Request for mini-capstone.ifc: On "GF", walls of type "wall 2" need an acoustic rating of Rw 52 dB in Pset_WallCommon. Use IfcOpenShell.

First a look at what the model holds.

```python
import ifcopenshell
import ifcopenshell.util.element

model = ifcopenshell.open("mini-capstone.ifc")
print(model.schema)
storey = next(s for s in model.by_type("IfcBuildingStorey") if s.Name == "GF")
walls = [e for e in ifcopenshell.util.element.get_decomposition(storey) if e.is_a("IfcWall")]
seen = {}
for e in walls:
    element_type = ifcopenshell.util.element.get_type(e)
    key = (element_type.Name if element_type != e and element_type else None, ifcopenshell.util.element.get_pset(e, "Pset_WallCommon", "AcousticRating"))
    seen[key] = seen.get(key, 0) + 1
for (name, value), count in sorted(seen.items(), key=str):
    print(count, "x", name, "|", value)
```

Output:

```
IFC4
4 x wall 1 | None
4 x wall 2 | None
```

```python
import ifcopenshell
import ifcopenshell.api.pset
import ifcopenshell.util.element

model = ifcopenshell.open("mini-capstone.ifc")

storey = next(s for s in model.by_type("IfcBuildingStorey") if s.Name == "GF")
walls = [e for e in ifcopenshell.util.element.get_decomposition(storey) if e.is_a("IfcWall")]

count = 0
for e in walls:
    element_type = ifcopenshell.util.element.get_type(e)
    if element_type in (None, e) or element_type.Name != "wall 2":
        continue
    # add_pset returns the element's existing set when there is one.
    pset = ifcopenshell.api.pset.add_pset(model, product=e, name="Pset_WallCommon")
    ifcopenshell.api.pset.edit_pset(model, pset=pset, properties={"AcousticRating": "Rw 52 dB"})
    count += 1

print(count, "walls updated")

model.write("mini-capstone_v2.ifc")
```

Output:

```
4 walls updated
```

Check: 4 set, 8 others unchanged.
